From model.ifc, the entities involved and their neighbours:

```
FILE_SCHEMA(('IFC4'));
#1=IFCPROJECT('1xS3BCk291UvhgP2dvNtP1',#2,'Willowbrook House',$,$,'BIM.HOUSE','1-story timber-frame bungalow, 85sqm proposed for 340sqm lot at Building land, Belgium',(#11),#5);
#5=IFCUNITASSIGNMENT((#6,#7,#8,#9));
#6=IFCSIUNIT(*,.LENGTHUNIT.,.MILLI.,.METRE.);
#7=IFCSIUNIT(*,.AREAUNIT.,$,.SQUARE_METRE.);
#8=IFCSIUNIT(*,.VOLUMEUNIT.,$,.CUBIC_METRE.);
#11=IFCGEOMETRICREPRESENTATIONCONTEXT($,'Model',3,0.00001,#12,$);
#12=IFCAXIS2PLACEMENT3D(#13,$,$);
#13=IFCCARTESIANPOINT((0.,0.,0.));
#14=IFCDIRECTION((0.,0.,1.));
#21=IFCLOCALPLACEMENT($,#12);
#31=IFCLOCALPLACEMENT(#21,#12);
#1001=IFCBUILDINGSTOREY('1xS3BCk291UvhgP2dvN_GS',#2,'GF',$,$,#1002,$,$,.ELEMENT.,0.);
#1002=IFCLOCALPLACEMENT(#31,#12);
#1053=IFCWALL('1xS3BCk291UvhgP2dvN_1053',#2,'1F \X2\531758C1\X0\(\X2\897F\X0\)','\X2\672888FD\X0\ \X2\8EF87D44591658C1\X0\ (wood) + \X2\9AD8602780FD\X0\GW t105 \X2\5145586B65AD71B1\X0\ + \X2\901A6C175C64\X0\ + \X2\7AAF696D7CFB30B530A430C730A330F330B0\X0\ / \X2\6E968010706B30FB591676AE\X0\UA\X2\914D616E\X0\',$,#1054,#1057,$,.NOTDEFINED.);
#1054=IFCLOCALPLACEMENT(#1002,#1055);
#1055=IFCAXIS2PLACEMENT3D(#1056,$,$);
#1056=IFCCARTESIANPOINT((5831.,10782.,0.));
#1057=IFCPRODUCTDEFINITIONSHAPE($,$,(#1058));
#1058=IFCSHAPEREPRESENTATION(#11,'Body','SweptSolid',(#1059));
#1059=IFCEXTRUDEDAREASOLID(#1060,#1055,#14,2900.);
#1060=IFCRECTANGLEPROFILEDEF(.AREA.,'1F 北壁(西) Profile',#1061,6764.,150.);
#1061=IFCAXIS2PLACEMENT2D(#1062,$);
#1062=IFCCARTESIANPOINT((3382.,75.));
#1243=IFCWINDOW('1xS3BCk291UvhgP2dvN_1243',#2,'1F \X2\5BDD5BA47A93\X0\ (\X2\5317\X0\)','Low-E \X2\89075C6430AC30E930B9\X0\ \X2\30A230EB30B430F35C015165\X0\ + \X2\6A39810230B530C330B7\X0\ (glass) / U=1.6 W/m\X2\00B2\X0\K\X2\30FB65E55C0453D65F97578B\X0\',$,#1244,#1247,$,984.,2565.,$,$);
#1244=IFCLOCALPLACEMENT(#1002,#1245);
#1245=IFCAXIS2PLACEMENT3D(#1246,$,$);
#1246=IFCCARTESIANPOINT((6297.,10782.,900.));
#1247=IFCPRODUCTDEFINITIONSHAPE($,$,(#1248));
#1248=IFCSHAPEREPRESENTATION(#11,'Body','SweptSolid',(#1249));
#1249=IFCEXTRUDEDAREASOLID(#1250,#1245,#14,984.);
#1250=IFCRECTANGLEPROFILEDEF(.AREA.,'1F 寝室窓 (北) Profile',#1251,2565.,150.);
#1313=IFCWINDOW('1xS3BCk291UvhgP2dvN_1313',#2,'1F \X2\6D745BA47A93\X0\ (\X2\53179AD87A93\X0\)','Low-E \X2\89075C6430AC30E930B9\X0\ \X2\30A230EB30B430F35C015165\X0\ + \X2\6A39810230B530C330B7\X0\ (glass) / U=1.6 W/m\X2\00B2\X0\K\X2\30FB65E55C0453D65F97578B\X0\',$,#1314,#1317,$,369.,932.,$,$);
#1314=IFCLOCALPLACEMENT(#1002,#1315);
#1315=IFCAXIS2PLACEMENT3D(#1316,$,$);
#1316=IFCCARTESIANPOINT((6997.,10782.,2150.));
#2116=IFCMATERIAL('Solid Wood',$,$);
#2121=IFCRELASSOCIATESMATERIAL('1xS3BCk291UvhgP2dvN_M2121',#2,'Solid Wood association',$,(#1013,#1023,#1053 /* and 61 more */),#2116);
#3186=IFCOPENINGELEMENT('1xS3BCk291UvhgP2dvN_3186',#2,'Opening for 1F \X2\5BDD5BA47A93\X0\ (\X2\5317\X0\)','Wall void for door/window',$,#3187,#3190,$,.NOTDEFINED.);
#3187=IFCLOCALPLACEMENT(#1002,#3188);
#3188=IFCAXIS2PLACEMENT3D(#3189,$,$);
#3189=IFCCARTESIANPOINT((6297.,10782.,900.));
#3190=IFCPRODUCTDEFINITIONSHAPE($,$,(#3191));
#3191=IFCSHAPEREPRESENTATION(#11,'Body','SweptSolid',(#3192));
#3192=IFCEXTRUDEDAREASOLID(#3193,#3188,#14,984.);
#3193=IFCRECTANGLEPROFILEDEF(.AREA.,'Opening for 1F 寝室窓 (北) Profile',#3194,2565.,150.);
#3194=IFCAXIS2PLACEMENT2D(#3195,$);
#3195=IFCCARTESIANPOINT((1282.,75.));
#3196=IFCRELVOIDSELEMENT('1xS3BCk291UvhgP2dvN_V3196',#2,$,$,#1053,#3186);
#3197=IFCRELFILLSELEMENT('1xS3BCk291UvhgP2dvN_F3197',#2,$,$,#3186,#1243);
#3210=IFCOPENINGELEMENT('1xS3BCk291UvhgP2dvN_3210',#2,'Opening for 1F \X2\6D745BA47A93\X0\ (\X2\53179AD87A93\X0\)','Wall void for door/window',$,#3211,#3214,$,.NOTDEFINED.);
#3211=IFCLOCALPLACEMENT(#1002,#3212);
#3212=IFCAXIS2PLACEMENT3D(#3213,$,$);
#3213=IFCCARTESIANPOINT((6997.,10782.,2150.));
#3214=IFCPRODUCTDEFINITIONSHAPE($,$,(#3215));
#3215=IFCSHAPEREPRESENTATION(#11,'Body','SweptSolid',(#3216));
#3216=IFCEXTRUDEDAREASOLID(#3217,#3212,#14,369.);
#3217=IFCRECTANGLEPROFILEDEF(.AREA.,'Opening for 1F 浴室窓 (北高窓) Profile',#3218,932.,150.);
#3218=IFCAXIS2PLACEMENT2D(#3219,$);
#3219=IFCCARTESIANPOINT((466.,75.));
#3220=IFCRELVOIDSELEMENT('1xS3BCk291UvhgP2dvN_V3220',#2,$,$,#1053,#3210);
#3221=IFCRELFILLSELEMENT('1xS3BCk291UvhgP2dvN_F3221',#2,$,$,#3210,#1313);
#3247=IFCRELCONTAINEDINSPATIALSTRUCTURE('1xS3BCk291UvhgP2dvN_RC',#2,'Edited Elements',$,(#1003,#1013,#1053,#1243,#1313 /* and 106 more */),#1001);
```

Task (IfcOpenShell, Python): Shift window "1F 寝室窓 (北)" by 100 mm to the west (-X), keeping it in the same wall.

```python
import ifcopenshell
import ifcopenshell.api.geometry
import ifcopenshell.util.placement

model = ifcopenshell.open("model.ifc")

window = model.by_id(1243)
opening = window.FillsVoids[0].RelatingOpeningElement
wall = opening.VoidsElements[0].RelatingBuildingElement

wall_matrix = ifcopenshell.util.placement.get_local_placement(wall.ObjectPlacement)
shift = wall_matrix[:3, 0] * -100.0
before = ifcopenshell.util.placement.get_local_placement(window.ObjectPlacement)[:3, 3].copy()

# The window is not placed relative to its opening, so move both.
for product in (opening, window):
    matrix = ifcopenshell.util.placement.get_local_placement(product.ObjectPlacement)
    matrix[:3, 3] += shift
    ifcopenshell.api.geometry.edit_object_placement(model, product=product, matrix=matrix, is_si=False)

after = ifcopenshell.util.placement.get_local_placement(window.ObjectPlacement)[:3, 3]
print("window moved by", (after - before).round(3) + 0.0)

model.write("model_v2.ifc")
```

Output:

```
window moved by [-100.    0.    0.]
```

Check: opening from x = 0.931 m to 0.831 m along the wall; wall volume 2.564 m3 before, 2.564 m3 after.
